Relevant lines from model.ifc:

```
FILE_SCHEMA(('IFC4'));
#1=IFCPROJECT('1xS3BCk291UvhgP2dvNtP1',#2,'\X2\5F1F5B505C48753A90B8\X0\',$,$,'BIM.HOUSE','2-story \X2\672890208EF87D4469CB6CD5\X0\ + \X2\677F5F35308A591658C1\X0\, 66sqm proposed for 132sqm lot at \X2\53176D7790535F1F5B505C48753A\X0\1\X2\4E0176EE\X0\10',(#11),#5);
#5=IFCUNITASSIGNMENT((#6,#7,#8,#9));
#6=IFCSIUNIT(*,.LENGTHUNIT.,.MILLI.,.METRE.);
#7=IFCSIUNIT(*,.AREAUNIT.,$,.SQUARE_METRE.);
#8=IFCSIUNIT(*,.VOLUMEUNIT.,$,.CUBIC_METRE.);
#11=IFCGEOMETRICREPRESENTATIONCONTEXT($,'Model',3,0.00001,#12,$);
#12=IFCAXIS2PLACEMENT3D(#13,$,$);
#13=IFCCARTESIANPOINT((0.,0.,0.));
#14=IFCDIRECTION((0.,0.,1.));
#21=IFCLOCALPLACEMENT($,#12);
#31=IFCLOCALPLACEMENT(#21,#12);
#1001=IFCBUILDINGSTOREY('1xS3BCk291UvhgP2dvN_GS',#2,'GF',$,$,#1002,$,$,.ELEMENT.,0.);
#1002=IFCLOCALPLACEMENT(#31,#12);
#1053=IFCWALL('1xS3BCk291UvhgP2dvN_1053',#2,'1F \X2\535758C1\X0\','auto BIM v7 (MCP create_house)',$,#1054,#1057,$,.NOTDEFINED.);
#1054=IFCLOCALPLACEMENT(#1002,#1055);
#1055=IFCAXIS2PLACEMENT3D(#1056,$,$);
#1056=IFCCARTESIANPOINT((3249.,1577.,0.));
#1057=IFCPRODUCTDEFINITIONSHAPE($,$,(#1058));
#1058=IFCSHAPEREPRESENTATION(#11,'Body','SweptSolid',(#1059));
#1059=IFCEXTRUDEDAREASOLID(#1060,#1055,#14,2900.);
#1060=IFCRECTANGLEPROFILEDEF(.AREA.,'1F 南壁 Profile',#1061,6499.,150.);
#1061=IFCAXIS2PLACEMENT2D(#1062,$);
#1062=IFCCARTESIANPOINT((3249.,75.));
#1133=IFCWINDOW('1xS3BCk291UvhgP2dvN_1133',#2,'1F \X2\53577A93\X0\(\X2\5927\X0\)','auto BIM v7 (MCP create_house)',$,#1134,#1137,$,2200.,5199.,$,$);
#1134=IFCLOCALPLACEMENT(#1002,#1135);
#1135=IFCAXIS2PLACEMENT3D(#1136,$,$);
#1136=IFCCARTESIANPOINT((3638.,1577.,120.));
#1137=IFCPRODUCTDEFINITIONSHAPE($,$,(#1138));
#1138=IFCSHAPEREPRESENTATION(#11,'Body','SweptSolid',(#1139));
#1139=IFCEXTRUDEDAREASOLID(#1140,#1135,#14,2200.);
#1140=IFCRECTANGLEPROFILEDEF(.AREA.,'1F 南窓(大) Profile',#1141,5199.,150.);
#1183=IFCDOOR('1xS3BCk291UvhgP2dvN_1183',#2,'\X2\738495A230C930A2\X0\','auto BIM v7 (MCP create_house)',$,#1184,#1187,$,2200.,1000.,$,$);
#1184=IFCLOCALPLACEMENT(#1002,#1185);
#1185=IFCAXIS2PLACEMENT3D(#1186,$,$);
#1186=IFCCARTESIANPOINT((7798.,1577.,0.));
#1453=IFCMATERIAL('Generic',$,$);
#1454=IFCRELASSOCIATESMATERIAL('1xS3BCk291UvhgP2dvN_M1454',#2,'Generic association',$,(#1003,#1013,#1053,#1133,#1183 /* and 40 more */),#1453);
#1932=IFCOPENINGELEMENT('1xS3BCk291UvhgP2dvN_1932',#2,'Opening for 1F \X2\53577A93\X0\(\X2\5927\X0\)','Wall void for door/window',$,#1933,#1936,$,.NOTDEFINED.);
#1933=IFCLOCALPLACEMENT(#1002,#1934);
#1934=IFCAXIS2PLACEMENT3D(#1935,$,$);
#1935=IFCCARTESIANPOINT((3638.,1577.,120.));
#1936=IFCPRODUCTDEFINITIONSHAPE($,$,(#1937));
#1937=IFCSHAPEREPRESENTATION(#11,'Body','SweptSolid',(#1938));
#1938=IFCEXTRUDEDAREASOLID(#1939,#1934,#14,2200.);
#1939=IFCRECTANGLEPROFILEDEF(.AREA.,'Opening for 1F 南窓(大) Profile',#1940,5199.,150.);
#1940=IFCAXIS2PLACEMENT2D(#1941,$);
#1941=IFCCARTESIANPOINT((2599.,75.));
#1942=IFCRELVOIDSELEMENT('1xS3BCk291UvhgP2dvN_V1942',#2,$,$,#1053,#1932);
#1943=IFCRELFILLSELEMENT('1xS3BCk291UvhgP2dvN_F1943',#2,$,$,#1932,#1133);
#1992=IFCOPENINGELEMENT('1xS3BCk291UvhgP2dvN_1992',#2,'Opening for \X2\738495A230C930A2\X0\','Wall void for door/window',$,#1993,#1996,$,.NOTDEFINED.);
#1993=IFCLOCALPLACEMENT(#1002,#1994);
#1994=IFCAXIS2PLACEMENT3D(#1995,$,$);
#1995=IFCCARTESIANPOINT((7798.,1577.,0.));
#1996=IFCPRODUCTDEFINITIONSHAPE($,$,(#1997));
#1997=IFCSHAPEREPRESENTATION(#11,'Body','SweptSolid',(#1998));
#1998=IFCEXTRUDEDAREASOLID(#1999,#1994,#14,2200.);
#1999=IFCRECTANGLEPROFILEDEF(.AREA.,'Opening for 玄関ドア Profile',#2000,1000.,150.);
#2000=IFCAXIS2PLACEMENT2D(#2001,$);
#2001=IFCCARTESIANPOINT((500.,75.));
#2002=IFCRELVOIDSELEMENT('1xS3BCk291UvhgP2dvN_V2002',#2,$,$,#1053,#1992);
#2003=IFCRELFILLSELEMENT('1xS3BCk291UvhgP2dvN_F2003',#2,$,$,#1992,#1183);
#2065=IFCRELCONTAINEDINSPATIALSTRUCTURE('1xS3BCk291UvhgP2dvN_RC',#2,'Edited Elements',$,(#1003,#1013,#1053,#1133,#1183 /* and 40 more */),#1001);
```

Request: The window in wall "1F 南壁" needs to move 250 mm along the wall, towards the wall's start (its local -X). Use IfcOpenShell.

```python
import ifcopenshell
import ifcopenshell.api.geometry
import ifcopenshell.util.placement
import ifcopenshell.util.unit

model = ifcopenshell.open("model.ifc")
unit_scale = ifcopenshell.util.unit.calculate_unit_scale(model)

window = model.by_guid("1xS3BCk291UvhgP2dvN_1133")
opening = window.FillsVoids[0].RelatingOpeningElement
wall = opening.VoidsElements[0].RelatingBuildingElement

wall_matrix = ifcopenshell.util.placement.get_local_placement(wall.ObjectPlacement)
shift = wall_matrix[:3, 0] * -0.25 / unit_scale
before = ifcopenshell.util.placement.get_local_placement(window.ObjectPlacement)[:3, 3].copy()

# The window is not placed relative to its opening, so move both.
for product in (opening, window):
    matrix = ifcopenshell.util.placement.get_local_placement(product.ObjectPlacement)
    matrix[:3, 3] += shift
    ifcopenshell.api.geometry.edit_object_placement(model, product=product, matrix=matrix, is_si=False)

after = ifcopenshell.util.placement.get_local_placement(window.ObjectPlacement)[:3, 3]
print("window moved by", (after - before).round(3) + 0.0)

model.write("model_v2.ifc")
```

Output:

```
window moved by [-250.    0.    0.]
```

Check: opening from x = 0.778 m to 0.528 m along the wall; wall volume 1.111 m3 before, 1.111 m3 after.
